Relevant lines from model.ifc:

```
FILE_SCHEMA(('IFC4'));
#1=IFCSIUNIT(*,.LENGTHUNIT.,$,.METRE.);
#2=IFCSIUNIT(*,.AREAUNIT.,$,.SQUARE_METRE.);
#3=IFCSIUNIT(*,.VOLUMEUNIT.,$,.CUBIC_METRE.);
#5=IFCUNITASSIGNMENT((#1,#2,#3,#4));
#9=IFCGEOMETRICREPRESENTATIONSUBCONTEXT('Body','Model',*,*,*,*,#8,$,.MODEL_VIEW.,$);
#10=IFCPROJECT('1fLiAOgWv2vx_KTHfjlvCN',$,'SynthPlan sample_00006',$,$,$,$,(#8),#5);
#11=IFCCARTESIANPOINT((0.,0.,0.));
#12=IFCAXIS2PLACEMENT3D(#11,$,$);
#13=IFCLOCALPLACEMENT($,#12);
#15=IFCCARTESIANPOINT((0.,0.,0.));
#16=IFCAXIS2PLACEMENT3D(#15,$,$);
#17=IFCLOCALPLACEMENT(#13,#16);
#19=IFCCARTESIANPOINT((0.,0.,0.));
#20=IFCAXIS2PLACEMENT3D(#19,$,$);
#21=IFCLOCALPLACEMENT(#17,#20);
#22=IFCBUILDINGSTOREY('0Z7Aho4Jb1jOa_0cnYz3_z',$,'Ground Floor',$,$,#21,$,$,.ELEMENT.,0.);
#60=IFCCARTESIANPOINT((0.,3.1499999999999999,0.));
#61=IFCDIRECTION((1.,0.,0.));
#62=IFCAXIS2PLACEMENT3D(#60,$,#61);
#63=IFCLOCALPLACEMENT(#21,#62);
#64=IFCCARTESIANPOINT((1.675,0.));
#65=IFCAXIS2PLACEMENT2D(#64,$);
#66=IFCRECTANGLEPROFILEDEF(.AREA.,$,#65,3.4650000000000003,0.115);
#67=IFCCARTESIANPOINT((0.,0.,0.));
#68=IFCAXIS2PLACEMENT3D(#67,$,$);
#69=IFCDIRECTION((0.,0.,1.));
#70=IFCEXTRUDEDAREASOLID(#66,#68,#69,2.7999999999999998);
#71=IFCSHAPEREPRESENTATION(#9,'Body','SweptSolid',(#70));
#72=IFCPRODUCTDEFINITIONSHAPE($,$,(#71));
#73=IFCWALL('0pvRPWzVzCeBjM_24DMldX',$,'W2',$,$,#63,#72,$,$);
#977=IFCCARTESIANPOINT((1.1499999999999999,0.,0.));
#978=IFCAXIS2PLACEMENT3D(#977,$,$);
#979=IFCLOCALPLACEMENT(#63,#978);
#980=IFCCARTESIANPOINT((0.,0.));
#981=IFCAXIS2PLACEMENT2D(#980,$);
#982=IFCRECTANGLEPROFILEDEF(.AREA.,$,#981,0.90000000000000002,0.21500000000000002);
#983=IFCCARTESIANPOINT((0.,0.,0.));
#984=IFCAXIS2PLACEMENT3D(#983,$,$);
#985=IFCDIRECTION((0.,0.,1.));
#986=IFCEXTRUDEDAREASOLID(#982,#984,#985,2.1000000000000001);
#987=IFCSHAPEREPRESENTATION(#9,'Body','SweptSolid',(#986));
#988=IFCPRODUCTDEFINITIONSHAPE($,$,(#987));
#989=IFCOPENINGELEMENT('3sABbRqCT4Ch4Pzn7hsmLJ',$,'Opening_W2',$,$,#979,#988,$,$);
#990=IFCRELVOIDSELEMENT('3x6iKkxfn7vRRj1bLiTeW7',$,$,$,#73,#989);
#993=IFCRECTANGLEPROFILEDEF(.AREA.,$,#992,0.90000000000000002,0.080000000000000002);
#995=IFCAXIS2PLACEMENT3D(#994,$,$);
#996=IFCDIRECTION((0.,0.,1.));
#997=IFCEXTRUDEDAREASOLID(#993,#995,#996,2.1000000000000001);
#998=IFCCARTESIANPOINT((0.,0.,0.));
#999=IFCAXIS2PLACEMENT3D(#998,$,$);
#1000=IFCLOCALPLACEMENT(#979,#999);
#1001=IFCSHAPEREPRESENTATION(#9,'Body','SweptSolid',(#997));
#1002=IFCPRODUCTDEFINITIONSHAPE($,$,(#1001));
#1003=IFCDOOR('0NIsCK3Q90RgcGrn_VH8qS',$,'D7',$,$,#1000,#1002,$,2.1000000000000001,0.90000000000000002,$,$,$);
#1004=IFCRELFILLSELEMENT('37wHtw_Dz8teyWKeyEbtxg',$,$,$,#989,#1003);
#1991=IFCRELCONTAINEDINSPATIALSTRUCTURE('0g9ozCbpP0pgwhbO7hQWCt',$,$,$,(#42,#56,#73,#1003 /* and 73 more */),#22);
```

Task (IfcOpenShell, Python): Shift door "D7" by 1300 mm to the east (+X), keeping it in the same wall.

```python
import ifcopenshell
import ifcopenshell.api.geometry
import ifcopenshell.util.placement
import ifcopenshell.util.unit

model = ifcopenshell.open("model.ifc")
unit_scale = ifcopenshell.util.unit.calculate_unit_scale(model)

door = model.by_id(1003)
opening = door.FillsVoids[0].RelatingOpeningElement
wall = opening.VoidsElements[0].RelatingBuildingElement

wall_matrix = ifcopenshell.util.placement.get_local_placement(wall.ObjectPlacement)
shift = wall_matrix[:3, 0] * 1.3 / unit_scale
before = ifcopenshell.util.placement.get_local_placement(door.ObjectPlacement)[:3, 3].copy()

# The door is placed relative to its opening, so it follows when the opening moves.
matrix = ifcopenshell.util.placement.get_local_placement(opening.ObjectPlacement)
matrix[:3, 3] += shift
ifcopenshell.api.geometry.edit_object_placement(
    model, product=opening, matrix=matrix, is_si=False, should_transform_children=True
)

after = ifcopenshell.util.placement.get_local_placement(door.ObjectPlacement)[:3, 3]
print("door moved by", (after - before).round(3) + 0.0)

model.write("model_v2.ifc")
```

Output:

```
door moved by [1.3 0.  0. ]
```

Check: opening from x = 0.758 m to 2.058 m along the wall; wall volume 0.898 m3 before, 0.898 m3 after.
